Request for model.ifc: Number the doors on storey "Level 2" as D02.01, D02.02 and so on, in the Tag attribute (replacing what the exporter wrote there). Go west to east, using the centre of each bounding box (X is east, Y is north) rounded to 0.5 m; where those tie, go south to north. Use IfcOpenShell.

First a look at what the model holds.

```python
import ifcopenshell
import ifcopenshell.util.element
import ifcopenshell.util.placement

model = ifcopenshell.open("model.ifc")
print(model.schema)
storey = next(s for s in model.by_type("IfcBuildingStorey") if s.Name == "Level 2")
doors = [e for e in ifcopenshell.util.element.get_decomposition(storey) if e.is_a("IfcDoor")]
for e in sorted(doors, key=lambda e: e.id()):
    origin = ifcopenshell.util.placement.get_local_placement(e.ObjectPlacement)[:3, 3]
    print(e.id(), e.Tag, e.Name, origin.round(2) + 0.0, sep=" | ")
```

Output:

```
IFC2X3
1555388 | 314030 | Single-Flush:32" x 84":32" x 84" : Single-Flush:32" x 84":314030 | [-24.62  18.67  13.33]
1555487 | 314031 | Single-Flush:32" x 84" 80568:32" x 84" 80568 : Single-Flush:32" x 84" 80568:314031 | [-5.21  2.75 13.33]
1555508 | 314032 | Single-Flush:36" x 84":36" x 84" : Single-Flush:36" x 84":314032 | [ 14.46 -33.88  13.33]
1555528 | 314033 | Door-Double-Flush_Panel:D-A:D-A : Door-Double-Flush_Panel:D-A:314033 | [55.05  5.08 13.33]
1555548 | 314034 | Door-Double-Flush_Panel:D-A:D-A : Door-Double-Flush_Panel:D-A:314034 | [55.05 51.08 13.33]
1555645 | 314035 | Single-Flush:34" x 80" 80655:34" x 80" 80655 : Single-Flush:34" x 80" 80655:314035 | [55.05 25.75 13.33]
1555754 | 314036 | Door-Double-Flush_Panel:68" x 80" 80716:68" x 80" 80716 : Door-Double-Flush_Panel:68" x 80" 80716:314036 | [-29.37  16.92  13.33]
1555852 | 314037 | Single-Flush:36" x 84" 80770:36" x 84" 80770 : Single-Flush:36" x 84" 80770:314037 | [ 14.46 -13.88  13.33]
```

```python
import ifcopenshell
import ifcopenshell.geom
import ifcopenshell.util.element
import ifcopenshell.util.shape

model = ifcopenshell.open("model.ifc")
settings = ifcopenshell.geom.settings()
settings.set("use-world-coords", True)


def centre(element):
    shape = ifcopenshell.geom.create_shape(settings, element)
    return ifcopenshell.util.shape.get_bbox_centroid(shape.geometry)


storey = next(s for s in model.by_type("IfcBuildingStorey") if s.Name == "Level 2")
doors = [e for e in ifcopenshell.util.element.get_decomposition(storey) if e.is_a("IfcDoor")]

# Insertion points can sit at a corner or the storey origin, so sort by the geometry (in metres).
centres = {e: centre(e) for e in doors}
doors.sort(key=lambda e: (round(centres[e][0] / 0.5), centres[e][1]))

for i, e in enumerate(doors, start=1):
    number = f"D02.{i:02d}"
    e.Tag = number
    print(e.id(), number)

model.write("model-out.ifc")
```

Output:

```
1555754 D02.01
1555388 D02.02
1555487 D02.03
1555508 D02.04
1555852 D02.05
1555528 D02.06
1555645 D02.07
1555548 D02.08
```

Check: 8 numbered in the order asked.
